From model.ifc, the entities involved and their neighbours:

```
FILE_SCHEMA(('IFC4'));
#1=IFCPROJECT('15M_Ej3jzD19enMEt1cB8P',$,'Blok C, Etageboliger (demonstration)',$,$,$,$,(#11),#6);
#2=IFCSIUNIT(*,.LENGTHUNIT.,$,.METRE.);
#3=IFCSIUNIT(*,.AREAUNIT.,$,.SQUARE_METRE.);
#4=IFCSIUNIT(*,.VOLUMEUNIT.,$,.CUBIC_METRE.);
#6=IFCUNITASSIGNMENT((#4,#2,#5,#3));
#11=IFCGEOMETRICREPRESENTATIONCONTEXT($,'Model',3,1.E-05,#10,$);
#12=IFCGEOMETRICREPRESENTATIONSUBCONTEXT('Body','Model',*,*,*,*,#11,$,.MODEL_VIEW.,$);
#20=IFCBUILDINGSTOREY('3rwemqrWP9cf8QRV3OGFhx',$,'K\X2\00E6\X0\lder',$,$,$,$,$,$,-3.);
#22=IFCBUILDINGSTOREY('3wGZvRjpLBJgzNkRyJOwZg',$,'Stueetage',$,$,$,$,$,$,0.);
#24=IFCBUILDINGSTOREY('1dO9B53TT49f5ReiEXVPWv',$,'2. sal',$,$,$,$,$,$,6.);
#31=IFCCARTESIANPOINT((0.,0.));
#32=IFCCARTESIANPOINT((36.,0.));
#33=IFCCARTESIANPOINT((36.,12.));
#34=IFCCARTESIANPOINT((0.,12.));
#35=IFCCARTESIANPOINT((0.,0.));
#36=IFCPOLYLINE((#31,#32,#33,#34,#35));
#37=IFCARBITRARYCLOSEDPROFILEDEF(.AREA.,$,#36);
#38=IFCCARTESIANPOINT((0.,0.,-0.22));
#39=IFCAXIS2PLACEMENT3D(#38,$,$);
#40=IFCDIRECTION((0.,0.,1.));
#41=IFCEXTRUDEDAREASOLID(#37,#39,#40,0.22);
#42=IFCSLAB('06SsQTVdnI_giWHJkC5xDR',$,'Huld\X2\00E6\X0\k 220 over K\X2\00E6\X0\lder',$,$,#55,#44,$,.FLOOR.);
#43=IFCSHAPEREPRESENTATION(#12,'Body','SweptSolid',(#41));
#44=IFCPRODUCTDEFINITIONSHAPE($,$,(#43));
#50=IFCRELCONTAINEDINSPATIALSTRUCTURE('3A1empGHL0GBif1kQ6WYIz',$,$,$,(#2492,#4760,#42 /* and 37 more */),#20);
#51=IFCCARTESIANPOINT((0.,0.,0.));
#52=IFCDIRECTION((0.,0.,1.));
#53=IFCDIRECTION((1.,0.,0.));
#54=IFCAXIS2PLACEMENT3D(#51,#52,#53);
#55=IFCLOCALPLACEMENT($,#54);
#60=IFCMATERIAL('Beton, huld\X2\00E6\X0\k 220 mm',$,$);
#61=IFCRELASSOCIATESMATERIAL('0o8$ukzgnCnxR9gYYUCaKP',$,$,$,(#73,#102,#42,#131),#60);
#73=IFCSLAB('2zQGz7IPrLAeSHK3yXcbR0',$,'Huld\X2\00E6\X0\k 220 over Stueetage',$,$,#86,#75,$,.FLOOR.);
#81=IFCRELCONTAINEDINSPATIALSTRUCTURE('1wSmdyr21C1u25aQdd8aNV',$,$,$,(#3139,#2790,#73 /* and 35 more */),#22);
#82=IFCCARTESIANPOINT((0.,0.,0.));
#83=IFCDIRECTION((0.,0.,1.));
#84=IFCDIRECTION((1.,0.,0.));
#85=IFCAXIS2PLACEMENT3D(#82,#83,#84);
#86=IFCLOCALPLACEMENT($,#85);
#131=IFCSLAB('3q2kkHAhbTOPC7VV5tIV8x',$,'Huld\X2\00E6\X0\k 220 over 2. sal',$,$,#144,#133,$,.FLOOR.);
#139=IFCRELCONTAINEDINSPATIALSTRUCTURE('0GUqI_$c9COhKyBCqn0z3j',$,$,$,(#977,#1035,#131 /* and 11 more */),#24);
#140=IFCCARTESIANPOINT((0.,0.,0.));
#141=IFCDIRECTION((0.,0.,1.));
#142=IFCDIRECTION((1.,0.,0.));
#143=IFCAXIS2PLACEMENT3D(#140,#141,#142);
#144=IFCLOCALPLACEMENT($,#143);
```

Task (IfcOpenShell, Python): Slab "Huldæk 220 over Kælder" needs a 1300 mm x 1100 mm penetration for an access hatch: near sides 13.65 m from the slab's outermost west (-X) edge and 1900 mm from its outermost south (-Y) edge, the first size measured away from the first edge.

```python
import numpy as np
import ifcopenshell
import ifcopenshell.api.feature
import ifcopenshell.api.geometry
import ifcopenshell.api.root
import ifcopenshell.geom
import ifcopenshell.util.placement
import ifcopenshell.util.representation
import ifcopenshell.util.shape
import ifcopenshell.util.unit

model = ifcopenshell.open("model.ifc")
unit_scale = ifcopenshell.util.unit.calculate_unit_scale(model)
settings = ifcopenshell.geom.settings()


def volume(element):
    """Net volume in cubic metres, openings subtracted."""
    shape = ifcopenshell.geom.create_shape(settings, element)
    return ifcopenshell.util.shape.get_volume(shape.geometry)


slab = model.by_guid("06SsQTVdnI_giWHJkC5xDR")
before = volume(slab)

# Extent in the slab's own axes, in metres. The edges named are its -X and -Y sides.
slab_shape = ifcopenshell.geom.create_shape(settings, slab)
vertices = ifcopenshell.util.shape.get_vertices(slab_shape.geometry)
x_min, y_min, bottom = vertices.min(axis=0)
top = vertices[:, 2].max()

opening = ifcopenshell.api.root.create_entity(model, ifc_class="IfcOpeningElement", name="Access hatch opening", predefined_type="OPENING")
context = ifcopenshell.util.representation.get_context(model, "Model", "Body", "MODEL_VIEW")
width, depth = 1.3, 1.1
outline = [(0.0, 0.0), (width, 0.0), (width, depth), (0.0, depth), (0.0, 0.0)]
# Overshoot both faces by 50 mm so the cut is clean.
shape = ifcopenshell.api.geometry.add_slab_representation(
    model, context=context, depth=top - bottom + 0.1, polyline=outline
)
ifcopenshell.api.geometry.assign_representation(model, product=opening, representation=shape)

matrix = ifcopenshell.util.placement.get_local_placement(slab.ObjectPlacement)
matrix[:, 3] = matrix @ np.append(np.array([x_min + 13.65, y_min + 1.9, bottom - 0.05]) / unit_scale, 1.0)
ifcopenshell.api.geometry.edit_object_placement(model, product=opening, matrix=matrix, is_si=False)
ifcopenshell.api.feature.add_feature(model, feature=opening, element=slab)

after = volume(slab)

print(f"slab volume {before:.3f} -> {after:.3f} m3")

model.write("model_v2.ifc")
```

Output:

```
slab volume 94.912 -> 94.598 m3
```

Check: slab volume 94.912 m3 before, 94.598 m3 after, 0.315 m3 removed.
